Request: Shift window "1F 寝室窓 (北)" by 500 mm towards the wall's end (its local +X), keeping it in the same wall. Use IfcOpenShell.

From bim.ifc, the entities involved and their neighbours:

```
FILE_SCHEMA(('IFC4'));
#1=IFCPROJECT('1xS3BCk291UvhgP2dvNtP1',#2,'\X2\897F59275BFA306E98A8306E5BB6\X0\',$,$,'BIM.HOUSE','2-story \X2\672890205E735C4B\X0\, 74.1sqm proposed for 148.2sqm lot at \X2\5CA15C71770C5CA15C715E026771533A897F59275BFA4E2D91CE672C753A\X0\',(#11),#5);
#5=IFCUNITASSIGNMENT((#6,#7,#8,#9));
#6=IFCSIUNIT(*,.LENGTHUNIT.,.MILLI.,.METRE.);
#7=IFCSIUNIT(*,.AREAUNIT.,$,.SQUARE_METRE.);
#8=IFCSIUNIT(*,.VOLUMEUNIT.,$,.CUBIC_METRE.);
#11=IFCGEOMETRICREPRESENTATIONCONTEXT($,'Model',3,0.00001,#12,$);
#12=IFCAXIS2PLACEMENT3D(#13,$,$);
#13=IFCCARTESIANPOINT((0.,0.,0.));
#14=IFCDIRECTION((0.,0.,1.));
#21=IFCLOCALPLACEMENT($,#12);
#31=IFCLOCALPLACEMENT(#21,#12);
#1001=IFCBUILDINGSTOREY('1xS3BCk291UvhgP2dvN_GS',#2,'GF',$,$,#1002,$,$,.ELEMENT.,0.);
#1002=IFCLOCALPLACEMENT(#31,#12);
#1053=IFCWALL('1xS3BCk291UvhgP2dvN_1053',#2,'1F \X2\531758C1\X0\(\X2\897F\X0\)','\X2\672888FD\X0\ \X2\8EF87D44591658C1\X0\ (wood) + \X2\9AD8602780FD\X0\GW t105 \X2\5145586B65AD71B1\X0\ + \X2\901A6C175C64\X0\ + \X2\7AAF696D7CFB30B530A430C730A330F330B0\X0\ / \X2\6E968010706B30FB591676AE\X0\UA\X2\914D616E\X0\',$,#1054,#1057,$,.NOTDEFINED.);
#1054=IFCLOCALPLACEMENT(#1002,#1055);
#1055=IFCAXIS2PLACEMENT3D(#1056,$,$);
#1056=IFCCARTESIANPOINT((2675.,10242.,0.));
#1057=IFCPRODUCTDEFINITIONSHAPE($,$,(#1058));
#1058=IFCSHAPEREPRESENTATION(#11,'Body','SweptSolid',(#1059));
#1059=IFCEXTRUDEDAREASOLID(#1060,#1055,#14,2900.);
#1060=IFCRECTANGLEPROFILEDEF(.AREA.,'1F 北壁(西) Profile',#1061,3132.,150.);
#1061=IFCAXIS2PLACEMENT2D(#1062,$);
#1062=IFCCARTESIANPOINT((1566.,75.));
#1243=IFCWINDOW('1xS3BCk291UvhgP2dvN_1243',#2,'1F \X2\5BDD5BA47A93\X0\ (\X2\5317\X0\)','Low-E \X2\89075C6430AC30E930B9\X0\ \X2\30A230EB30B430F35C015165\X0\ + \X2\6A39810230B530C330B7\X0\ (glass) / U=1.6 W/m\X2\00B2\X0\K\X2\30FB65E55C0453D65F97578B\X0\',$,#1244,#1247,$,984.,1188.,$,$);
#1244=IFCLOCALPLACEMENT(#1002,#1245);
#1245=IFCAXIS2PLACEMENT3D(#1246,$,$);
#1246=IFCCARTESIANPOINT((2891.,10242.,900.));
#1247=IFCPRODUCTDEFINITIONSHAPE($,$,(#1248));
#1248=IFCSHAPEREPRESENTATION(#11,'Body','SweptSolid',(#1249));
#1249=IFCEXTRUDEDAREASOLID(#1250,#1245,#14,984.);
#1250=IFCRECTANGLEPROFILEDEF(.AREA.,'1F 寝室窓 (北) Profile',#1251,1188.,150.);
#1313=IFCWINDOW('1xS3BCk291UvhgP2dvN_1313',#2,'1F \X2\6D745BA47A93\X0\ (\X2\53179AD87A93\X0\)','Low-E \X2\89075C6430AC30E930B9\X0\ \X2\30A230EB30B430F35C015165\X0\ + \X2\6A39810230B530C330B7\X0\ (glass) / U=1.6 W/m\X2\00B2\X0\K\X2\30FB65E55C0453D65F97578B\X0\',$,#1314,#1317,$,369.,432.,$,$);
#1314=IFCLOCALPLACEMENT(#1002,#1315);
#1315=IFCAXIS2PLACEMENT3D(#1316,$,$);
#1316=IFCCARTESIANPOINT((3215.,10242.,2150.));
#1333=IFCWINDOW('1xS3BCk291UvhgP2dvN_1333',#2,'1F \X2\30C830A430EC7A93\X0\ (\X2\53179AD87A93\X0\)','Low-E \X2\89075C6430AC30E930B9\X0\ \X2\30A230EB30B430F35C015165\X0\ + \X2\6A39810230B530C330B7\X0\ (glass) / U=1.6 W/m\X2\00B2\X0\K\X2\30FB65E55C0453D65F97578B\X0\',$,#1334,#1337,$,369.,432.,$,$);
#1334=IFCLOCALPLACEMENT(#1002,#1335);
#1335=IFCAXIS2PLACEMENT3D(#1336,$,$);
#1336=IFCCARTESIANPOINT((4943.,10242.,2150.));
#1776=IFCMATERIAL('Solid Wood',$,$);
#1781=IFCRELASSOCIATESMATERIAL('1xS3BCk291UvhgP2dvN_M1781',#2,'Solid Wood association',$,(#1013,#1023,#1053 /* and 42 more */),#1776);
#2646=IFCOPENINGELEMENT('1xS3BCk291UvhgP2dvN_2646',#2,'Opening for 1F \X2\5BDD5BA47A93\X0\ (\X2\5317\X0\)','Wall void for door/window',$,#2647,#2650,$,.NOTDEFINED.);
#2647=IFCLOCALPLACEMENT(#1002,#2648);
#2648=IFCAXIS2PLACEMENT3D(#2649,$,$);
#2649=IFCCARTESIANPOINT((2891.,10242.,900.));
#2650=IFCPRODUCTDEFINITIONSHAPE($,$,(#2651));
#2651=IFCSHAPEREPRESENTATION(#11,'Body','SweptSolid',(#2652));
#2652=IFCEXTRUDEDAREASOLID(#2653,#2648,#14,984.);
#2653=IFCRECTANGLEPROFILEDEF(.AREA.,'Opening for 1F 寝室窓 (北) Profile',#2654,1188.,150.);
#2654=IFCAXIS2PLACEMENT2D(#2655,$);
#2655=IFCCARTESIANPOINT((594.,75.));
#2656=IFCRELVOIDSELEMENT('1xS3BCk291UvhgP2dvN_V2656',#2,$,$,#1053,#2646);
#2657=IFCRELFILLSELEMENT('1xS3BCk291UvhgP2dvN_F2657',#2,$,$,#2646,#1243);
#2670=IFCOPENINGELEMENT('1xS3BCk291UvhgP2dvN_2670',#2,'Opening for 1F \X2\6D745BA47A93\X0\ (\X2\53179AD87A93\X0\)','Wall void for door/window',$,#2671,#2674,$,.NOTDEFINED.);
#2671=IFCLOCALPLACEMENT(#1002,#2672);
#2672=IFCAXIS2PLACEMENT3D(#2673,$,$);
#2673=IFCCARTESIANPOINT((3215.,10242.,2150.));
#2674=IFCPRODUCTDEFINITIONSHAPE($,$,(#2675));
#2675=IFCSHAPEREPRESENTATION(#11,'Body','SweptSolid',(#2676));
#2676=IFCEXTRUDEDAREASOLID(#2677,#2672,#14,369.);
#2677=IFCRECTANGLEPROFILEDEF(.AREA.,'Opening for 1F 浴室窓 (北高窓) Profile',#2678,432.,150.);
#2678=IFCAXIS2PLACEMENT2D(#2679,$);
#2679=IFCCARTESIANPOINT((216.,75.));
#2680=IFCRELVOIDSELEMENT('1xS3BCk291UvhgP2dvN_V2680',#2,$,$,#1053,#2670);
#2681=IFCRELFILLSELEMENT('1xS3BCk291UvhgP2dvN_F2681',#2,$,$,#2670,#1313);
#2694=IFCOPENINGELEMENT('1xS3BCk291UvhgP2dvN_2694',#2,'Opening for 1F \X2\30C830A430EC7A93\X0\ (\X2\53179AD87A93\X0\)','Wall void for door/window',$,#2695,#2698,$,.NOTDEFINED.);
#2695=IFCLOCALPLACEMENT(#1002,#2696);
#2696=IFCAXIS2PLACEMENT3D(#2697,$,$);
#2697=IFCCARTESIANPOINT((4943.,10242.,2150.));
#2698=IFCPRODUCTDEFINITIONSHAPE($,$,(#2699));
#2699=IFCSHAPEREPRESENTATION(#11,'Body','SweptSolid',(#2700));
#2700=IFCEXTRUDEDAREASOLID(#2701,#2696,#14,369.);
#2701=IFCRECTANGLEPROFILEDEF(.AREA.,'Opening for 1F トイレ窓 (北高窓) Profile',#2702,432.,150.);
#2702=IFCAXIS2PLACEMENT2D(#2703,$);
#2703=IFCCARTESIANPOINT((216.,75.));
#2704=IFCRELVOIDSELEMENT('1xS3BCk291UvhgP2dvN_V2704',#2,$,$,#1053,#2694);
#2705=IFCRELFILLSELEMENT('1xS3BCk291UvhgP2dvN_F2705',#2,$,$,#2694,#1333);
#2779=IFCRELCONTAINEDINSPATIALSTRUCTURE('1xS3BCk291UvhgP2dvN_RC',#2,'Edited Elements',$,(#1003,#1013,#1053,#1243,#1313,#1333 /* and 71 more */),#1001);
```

```python
import ifcopenshell
import ifcopenshell.api.geometry
import ifcopenshell.util.placement
import ifcopenshell.util.unit

model = ifcopenshell.open("bim.ifc")
unit_scale = ifcopenshell.util.unit.calculate_unit_scale(model)

window = model.by_guid("1xS3BCk291UvhgP2dvN_1243")
opening = window.FillsVoids[0].RelatingOpeningElement
wall = opening.VoidsElements[0].RelatingBuildingElement

wall_matrix = ifcopenshell.util.placement.get_local_placement(wall.ObjectPlacement)
shift = wall_matrix[:3, 0] * 0.5 / unit_scale
before = ifcopenshell.util.placement.get_local_placement(window.ObjectPlacement)[:3, 3].copy()

# The window is not placed relative to its opening, so move both.
for product in (opening, window):
    matrix = ifcopenshell.util.placement.get_local_placement(product.ObjectPlacement)
    matrix[:3, 3] += shift
    ifcopenshell.api.geometry.edit_object_placement(model, product=product, matrix=matrix, is_si=False)

after = ifcopenshell.util.placement.get_local_placement(window.ObjectPlacement)[:3, 3]
print("window moved by", (after - before).round(3) + 0.0)

model.write("bim_rev.ifc")
```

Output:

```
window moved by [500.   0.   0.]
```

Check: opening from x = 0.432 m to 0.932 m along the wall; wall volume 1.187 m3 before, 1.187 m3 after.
